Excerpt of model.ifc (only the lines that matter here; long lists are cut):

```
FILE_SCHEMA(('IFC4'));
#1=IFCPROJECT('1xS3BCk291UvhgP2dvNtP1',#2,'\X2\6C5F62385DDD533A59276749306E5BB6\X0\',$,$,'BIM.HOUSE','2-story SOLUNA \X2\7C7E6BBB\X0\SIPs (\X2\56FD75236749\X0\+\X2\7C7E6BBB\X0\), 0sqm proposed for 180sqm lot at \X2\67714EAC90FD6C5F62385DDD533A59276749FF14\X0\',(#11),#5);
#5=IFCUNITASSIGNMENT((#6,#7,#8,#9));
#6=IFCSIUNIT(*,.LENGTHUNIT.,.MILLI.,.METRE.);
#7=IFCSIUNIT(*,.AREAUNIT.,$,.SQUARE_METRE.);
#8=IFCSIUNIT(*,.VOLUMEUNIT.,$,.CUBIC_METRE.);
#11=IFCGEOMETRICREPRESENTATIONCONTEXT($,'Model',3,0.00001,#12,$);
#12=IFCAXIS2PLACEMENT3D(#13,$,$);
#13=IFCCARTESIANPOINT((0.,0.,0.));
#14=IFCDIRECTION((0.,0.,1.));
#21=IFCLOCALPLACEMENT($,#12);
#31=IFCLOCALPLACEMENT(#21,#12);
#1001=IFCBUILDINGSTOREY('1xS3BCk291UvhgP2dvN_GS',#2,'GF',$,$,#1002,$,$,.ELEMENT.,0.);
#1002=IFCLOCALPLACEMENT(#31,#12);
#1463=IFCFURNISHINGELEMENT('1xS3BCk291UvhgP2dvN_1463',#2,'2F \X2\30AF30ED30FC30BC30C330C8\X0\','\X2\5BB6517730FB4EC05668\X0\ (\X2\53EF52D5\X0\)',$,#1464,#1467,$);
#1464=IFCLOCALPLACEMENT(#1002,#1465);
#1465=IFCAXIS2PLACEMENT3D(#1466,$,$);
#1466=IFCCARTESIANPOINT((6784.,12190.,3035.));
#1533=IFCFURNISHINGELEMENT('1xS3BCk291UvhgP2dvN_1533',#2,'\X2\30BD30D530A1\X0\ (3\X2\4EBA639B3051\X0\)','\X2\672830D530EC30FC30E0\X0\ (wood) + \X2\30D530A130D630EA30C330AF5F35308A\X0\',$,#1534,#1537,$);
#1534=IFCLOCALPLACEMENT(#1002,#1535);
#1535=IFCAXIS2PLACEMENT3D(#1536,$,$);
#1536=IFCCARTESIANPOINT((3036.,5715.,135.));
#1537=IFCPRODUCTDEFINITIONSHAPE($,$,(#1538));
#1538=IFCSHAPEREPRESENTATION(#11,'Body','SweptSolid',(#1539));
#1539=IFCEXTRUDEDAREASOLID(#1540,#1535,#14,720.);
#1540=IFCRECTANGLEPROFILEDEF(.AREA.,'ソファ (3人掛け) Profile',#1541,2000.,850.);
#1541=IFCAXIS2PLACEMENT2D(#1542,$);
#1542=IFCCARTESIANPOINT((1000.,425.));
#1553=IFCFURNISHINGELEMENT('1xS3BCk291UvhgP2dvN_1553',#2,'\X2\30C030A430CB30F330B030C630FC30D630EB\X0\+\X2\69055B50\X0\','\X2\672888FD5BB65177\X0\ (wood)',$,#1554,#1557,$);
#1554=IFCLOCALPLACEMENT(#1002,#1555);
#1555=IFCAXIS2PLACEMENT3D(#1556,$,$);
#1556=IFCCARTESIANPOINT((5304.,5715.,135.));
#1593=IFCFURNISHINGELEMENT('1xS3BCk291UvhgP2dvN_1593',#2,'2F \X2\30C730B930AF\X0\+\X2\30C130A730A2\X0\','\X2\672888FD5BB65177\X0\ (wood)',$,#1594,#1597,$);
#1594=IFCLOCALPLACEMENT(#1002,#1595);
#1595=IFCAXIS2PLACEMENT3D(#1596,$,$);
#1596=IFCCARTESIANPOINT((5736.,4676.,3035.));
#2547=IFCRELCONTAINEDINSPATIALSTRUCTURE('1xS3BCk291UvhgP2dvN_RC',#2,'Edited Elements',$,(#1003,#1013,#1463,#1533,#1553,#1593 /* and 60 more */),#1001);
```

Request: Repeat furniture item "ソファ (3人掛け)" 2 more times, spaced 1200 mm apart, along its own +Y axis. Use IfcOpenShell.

```python
import ifcopenshell
import ifcopenshell.api.geometry
import ifcopenshell.api.root
import ifcopenshell.util.element
import ifcopenshell.util.placement
import ifcopenshell.util.unit

model = ifcopenshell.open("model.ifc")
unit_scale = ifcopenshell.util.unit.calculate_unit_scale(model)


def reuse_history(source, copy):
    """copy_class also copies each property set's owner history, people and application; keep the originals."""
    for rel in copy.IsDefinedBy:
        if rel.is_a("IfcRelDefinesByProperties") and (history := rel.RelatingPropertyDefinition.OwnerHistory):
            rel.RelatingPropertyDefinition.OwnerHistory = source.OwnerHistory
            ifcopenshell.util.element.remove_deep2(model, history)


source = model.by_guid("1xS3BCk291UvhgP2dvN_1533")
base = ifcopenshell.util.placement.get_local_placement(source.ObjectPlacement)
step = base[:3, 1] * 1.2 / unit_scale

for i in range(1, 3):
    copy = ifcopenshell.api.root.copy_class(model, product=source)
    copy.Representation = ifcopenshell.util.element.copy_deep(
        model, source.Representation, exclude=["IfcGeometricRepresentationContext", "IfcRepresentationMap"]
    )
    reuse_history(source, copy)
    matrix = base.copy()
    matrix[:3, 3] += i * step
    print("added at", matrix[:3, 3].round(3) + 0.0)
    ifcopenshell.api.geometry.edit_object_placement(model, product=copy, matrix=matrix, is_si=False)

model.write("model_v2.ifc")
```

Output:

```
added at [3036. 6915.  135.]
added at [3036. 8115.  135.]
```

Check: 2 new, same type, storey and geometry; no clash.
